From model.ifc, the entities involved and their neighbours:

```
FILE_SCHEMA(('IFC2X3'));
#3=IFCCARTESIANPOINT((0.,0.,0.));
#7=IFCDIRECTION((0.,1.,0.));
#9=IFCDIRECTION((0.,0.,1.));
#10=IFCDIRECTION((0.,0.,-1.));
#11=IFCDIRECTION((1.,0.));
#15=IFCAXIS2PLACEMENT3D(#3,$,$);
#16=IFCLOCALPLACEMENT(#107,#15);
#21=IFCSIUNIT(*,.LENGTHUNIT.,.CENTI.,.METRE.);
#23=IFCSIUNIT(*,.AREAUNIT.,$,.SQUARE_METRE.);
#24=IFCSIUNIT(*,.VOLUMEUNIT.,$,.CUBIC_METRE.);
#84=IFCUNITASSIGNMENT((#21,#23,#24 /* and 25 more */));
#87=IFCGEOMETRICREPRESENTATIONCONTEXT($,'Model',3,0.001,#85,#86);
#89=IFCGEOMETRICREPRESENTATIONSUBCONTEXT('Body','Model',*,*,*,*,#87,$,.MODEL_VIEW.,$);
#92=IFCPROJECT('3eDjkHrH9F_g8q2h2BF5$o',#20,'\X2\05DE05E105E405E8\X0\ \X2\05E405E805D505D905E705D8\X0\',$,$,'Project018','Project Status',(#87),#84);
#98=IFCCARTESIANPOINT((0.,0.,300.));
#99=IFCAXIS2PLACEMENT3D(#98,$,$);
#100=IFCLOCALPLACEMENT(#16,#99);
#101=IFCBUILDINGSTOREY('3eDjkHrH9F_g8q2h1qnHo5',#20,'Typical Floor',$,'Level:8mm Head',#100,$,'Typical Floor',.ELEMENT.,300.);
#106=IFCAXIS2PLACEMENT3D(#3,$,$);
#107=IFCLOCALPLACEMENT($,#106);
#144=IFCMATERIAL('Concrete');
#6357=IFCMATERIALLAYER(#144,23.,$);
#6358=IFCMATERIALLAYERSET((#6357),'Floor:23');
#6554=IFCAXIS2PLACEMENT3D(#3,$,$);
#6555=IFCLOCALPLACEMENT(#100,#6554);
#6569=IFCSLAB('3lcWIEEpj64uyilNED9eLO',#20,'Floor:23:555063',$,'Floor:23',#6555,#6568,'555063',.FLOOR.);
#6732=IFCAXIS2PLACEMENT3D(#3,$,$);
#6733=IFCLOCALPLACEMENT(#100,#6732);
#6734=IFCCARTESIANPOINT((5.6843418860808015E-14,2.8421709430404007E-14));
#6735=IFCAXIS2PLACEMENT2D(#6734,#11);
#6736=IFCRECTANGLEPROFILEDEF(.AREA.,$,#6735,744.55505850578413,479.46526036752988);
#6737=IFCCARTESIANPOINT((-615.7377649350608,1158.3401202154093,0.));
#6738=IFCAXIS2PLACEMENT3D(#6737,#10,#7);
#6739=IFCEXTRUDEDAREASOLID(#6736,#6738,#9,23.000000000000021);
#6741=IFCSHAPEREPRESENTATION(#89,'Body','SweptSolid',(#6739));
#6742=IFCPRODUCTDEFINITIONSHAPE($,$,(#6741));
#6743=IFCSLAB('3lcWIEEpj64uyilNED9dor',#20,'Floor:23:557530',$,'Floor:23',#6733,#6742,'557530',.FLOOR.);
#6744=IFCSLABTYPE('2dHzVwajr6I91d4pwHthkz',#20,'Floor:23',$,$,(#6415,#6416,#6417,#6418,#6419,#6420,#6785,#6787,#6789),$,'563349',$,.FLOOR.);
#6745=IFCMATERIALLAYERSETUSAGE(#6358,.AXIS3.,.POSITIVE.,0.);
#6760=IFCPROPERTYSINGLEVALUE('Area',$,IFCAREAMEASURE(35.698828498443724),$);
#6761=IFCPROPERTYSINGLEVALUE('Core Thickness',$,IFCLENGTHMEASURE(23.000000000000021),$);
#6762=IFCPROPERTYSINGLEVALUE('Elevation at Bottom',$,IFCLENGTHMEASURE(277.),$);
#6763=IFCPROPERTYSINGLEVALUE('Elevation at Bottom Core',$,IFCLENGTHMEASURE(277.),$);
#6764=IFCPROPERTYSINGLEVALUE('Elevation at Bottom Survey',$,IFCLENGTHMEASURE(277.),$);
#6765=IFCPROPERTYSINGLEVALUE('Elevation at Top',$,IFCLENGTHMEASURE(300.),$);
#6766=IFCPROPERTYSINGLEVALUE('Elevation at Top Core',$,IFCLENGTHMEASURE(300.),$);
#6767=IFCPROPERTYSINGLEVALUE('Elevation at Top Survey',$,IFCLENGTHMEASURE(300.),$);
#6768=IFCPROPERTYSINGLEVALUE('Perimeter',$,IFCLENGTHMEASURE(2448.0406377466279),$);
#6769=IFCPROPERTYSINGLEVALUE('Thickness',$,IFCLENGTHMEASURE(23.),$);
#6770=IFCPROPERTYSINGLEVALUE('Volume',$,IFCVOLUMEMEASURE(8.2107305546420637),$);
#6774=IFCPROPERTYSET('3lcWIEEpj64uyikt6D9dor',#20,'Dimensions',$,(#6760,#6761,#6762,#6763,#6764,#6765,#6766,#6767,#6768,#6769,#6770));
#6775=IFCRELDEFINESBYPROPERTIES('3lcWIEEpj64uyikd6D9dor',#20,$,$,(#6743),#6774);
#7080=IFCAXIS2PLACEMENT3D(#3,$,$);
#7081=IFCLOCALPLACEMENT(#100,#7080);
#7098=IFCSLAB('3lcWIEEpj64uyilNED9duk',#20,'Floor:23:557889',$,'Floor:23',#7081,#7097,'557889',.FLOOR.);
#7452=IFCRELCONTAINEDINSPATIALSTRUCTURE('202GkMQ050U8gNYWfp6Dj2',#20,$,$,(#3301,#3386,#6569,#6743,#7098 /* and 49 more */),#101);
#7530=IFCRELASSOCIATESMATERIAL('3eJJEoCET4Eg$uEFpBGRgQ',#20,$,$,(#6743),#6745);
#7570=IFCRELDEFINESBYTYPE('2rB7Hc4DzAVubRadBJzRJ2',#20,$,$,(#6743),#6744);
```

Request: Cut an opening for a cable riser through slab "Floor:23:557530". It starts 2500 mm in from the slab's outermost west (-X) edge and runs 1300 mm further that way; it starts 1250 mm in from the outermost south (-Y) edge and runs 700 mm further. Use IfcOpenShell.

```python
import numpy as np
import ifcopenshell
import ifcopenshell.api.feature
import ifcopenshell.api.geometry
import ifcopenshell.api.pset
import ifcopenshell.api.root
import ifcopenshell.geom
import ifcopenshell.util.element
import ifcopenshell.util.placement
import ifcopenshell.util.representation
import ifcopenshell.util.shape
import ifcopenshell.util.unit

model = ifcopenshell.open("model.ifc")
unit_scale = ifcopenshell.util.unit.calculate_unit_scale(model)
area_scale = ifcopenshell.util.unit.calculate_unit_scale(model, "AREAUNIT")
volume_scale = ifcopenshell.util.unit.calculate_unit_scale(model, "VOLUMEUNIT")
settings = ifcopenshell.geom.settings()


def volume(element):
    """Net volume in cubic metres, openings subtracted."""
    shape = ifcopenshell.geom.create_shape(settings, element)
    return ifcopenshell.util.shape.get_volume(shape.geometry)


slab = model.by_guid("3lcWIEEpj64uyilNED9dor")
before = volume(slab)

# Extent in the slab's own axes, in metres. The edges named are its -X and -Y sides.
slab_shape = ifcopenshell.geom.create_shape(settings, slab)
vertices = ifcopenshell.util.shape.get_vertices(slab_shape.geometry)
x_min, y_min, bottom = vertices.min(axis=0)
top = vertices[:, 2].max()

opening = ifcopenshell.api.root.create_entity(model, ifc_class="IfcOpeningElement", name="Cable riser opening")
context = ifcopenshell.util.representation.get_context(model, "Model", "Body", "MODEL_VIEW")
width, depth = 1.3, 0.7
outline = [(0.0, 0.0), (width, 0.0), (width, depth), (0.0, depth), (0.0, 0.0)]
# Overshoot both faces by 50 mm so the cut is clean.
shape = ifcopenshell.api.geometry.add_slab_representation(
    model, context=context, depth=top - bottom + 0.1, polyline=outline
)
ifcopenshell.api.geometry.assign_representation(model, product=opening, representation=shape)

matrix = ifcopenshell.util.placement.get_local_placement(slab.ObjectPlacement)
matrix[:, 3] = matrix @ np.append(np.array([x_min + 2.5, y_min + 1.25, bottom - 0.05]) / unit_scale, 1.0)
ifcopenshell.api.geometry.edit_object_placement(model, product=opening, matrix=matrix, is_si=False)
ifcopenshell.api.feature.add_feature(model, feature=opening, element=slab)

after = volume(slab)

# Update the slab's stored quantities.
pset = model.by_id(ifcopenshell.util.element.get_pset(slab, "Dimensions", should_inherit=False)["id"])
ifcopenshell.api.pset.edit_pset(model, pset=pset, properties={
    "Area": model.create_entity("IfcAreaMeasure", after / (top - bottom) / area_scale),
    "Volume": model.create_entity("IfcVolumeMeasure", after / volume_scale),
})

print(f"slab volume {before:.3f} -> {after:.3f} m3")

model.write("model_edited.ifc")
```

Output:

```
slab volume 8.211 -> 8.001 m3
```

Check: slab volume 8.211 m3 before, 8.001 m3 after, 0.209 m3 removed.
